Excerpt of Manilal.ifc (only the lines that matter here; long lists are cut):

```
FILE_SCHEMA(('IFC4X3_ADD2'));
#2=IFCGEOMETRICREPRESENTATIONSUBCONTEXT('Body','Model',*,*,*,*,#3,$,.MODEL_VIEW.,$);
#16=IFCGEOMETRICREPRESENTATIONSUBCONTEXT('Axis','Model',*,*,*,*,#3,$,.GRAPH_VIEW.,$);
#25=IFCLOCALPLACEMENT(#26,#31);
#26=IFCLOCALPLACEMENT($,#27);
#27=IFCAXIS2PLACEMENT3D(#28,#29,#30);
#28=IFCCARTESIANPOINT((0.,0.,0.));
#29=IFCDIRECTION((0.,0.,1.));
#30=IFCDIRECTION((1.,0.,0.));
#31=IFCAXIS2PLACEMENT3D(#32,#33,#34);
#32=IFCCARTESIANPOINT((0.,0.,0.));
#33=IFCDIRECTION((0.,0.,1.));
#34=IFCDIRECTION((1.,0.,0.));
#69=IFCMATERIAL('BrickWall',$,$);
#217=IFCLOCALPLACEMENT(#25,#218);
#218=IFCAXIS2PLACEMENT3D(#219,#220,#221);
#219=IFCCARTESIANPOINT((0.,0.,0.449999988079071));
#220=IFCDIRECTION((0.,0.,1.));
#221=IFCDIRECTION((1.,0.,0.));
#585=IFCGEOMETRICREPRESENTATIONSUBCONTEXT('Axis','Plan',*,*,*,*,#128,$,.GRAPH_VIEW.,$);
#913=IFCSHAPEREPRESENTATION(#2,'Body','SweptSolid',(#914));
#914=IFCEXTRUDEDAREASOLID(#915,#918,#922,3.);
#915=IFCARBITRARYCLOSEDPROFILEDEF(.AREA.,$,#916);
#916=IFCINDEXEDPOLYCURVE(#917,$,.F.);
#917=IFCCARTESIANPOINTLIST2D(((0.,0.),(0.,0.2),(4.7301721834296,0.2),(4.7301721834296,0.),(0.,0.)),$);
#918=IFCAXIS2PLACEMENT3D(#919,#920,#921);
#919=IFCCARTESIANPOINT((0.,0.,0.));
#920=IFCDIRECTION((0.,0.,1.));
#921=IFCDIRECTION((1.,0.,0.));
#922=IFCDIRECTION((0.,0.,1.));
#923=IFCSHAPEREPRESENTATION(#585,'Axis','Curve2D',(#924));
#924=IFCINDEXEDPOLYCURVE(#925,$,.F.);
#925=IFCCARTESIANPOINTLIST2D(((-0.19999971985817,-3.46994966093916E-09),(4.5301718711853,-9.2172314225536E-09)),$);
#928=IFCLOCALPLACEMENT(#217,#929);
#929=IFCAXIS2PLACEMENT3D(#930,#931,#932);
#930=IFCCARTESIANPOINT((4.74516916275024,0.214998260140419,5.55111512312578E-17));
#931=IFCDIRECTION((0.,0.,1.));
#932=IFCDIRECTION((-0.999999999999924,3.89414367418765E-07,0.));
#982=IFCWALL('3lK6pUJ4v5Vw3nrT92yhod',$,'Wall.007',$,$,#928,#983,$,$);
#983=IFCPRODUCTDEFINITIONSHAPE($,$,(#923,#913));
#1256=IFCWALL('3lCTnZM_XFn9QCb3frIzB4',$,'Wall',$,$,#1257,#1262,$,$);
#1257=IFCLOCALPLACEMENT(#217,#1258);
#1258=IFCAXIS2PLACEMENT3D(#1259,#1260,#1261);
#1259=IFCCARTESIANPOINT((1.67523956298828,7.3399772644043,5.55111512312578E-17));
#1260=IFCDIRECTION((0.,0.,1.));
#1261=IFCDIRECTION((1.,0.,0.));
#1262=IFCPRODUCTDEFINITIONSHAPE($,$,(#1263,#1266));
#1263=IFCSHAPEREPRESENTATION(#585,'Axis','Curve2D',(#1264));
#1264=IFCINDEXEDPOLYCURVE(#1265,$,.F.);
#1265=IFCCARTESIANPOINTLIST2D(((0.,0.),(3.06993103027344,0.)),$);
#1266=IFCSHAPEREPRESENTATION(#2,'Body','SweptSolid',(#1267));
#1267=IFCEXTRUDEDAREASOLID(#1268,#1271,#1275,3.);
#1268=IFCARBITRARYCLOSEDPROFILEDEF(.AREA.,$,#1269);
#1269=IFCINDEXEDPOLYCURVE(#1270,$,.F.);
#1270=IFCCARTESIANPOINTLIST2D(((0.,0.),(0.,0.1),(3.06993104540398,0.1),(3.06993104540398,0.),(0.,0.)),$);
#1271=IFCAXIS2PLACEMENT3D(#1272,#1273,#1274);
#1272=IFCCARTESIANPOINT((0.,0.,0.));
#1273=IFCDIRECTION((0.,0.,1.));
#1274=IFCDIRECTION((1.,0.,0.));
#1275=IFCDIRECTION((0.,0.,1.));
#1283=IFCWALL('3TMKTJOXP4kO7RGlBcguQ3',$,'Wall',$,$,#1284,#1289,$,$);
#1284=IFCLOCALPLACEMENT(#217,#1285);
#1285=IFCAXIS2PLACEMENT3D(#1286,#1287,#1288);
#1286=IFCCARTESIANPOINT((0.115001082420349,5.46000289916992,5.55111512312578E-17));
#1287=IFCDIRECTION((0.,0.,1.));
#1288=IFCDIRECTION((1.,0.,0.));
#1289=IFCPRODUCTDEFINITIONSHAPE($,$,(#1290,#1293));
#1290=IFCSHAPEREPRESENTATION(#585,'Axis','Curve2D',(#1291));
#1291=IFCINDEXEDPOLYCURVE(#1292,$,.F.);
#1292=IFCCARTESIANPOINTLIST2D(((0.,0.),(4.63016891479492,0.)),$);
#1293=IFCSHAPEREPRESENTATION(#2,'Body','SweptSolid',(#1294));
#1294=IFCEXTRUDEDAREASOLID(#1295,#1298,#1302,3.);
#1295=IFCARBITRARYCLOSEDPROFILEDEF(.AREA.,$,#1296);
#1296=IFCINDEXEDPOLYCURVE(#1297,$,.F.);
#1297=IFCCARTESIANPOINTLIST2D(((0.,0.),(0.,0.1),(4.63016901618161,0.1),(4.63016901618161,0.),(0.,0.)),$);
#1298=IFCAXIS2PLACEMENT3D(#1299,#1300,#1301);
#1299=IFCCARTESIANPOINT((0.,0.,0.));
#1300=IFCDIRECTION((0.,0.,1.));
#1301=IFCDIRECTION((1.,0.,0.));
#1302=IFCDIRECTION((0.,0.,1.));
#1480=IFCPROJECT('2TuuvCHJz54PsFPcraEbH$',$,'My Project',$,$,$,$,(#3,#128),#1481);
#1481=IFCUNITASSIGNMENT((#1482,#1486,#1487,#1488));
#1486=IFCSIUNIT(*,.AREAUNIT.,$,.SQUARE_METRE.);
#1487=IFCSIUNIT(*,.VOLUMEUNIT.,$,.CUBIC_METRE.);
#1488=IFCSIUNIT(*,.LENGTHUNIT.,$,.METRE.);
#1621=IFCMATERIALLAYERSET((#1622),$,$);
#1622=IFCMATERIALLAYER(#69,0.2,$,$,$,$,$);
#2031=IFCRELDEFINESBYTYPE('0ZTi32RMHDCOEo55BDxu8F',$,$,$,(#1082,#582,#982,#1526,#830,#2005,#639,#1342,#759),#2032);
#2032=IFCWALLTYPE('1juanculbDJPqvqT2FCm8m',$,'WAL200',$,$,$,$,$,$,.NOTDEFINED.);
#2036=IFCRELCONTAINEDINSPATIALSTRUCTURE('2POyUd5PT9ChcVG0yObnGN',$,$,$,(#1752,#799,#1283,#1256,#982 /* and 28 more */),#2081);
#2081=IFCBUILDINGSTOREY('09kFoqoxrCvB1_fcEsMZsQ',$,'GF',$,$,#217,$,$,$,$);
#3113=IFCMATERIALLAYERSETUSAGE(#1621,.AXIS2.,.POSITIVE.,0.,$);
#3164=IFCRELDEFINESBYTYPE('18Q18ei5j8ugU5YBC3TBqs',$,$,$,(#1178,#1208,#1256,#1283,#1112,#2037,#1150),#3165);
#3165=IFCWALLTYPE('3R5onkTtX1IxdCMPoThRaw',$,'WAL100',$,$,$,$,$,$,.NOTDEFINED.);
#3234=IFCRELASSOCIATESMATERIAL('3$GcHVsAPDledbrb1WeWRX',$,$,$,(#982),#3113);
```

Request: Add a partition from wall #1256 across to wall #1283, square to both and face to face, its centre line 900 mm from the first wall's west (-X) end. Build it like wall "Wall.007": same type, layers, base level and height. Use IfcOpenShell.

```python
import numpy as np
import ifcopenshell
import ifcopenshell.api.geometry
import ifcopenshell.api.material
import ifcopenshell.api.pset
import ifcopenshell.api.root
import ifcopenshell.api.spatial
import ifcopenshell.api.type
import ifcopenshell.geom
import ifcopenshell.util.element
import ifcopenshell.util.placement
import ifcopenshell.util.representation
import ifcopenshell.util.shape
import ifcopenshell.util.unit

model = ifcopenshell.open("Manilal.ifc")
unit_scale = ifcopenshell.util.unit.calculate_unit_scale(model)
settings = ifcopenshell.geom.settings()
settings.set("use-world-coords", True)

start_wall = model.by_guid("3lCTnZM_XFn9QCb3frIzB4")
end_wall = model.by_guid("3TMKTJOXP4kO7RGlBcguQ3")
like = model.by_guid("3lK6pUJ4v5Vw3nrT92yhod")
matrix = ifcopenshell.util.placement.get_local_placement(start_wall.ObjectPlacement)
matrix[:3, 3] *= unit_scale


def extent(element):
    """Bounding box in the first wall's axes, in metres."""
    shape = ifcopenshell.geom.create_shape(settings, element)
    points = (ifcopenshell.util.shape.get_vertices(shape.geometry) - matrix[:3, 3]) @ matrix[:3, :3]
    return points.min(axis=0), points.max(axis=0)


y_start = extent(start_wall)[0][1]
y_end = extent(end_wall)[1][1]
like_min, like_max = extent(like)
length, height = float(abs(y_end - y_start)), float(like_max[2] - like_min[2])
layer_set = ifcopenshell.util.element.get_material(like, should_skip_usage=True)
thickness = sum(layer.LayerThickness for layer in layer_set.MaterialLayers) * unit_scale

wall = ifcopenshell.api.root.create_entity(model, ifc_class="IfcWall", name="New partition")
storey = ifcopenshell.util.element.get_container(like)
ifcopenshell.api.spatial.assign_container(model, products=[wall], relating_structure=storey)
ifcopenshell.api.type.assign_type(
    model, related_objects=[wall], relating_type=ifcopenshell.util.element.get_type(like), should_map_representations=False
)
rel = ifcopenshell.api.material.assign_material(
    model, products=[wall], type="IfcMaterialLayerSetUsage", material=layer_set
)
rel.RelatingMaterial.OffsetFromReferenceLine = -thickness / 2 / unit_scale
pset = ifcopenshell.api.pset.add_pset(model, product=wall, name="Pset_WallCommon")
ifcopenshell.api.pset.edit_pset(model, pset=pset, properties={"IsExternal": False, "LoadBearing": False})

# The axis runs down the middle of the wall.
axis = ifcopenshell.api.geometry.add_axis_representation(
    model, context=ifcopenshell.util.representation.get_context(model, "Model", "Axis"), axis=[(0.0, 0.0), (length, 0.0)]
)
body = ifcopenshell.api.geometry.add_wall_representation(
    model,
    context=ifcopenshell.util.representation.get_context(model, "Model", "Body", "MODEL_VIEW"),
    length=length,
    height=height,
    thickness=thickness,
    offset=-thickness / 2,
)
for representation in (axis, body):
    ifcopenshell.api.geometry.assign_representation(model, product=wall, representation=representation)

placement = matrix @ ifcopenshell.util.placement.rotation(-90, "Z")
placement[:, 3] = matrix @ np.array([extent(start_wall)[0][0] + 0.9, y_start, like_min[2], 1.0])
ifcopenshell.api.geometry.edit_object_placement(model, product=wall, matrix=placement)

print(f"partition {length:.3f} m long, {height:.3f} m high, {thickness:.3f} m thick")

model.write("Manilal_edited.ifc")
```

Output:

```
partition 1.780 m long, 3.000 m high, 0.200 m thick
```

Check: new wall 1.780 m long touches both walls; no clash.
